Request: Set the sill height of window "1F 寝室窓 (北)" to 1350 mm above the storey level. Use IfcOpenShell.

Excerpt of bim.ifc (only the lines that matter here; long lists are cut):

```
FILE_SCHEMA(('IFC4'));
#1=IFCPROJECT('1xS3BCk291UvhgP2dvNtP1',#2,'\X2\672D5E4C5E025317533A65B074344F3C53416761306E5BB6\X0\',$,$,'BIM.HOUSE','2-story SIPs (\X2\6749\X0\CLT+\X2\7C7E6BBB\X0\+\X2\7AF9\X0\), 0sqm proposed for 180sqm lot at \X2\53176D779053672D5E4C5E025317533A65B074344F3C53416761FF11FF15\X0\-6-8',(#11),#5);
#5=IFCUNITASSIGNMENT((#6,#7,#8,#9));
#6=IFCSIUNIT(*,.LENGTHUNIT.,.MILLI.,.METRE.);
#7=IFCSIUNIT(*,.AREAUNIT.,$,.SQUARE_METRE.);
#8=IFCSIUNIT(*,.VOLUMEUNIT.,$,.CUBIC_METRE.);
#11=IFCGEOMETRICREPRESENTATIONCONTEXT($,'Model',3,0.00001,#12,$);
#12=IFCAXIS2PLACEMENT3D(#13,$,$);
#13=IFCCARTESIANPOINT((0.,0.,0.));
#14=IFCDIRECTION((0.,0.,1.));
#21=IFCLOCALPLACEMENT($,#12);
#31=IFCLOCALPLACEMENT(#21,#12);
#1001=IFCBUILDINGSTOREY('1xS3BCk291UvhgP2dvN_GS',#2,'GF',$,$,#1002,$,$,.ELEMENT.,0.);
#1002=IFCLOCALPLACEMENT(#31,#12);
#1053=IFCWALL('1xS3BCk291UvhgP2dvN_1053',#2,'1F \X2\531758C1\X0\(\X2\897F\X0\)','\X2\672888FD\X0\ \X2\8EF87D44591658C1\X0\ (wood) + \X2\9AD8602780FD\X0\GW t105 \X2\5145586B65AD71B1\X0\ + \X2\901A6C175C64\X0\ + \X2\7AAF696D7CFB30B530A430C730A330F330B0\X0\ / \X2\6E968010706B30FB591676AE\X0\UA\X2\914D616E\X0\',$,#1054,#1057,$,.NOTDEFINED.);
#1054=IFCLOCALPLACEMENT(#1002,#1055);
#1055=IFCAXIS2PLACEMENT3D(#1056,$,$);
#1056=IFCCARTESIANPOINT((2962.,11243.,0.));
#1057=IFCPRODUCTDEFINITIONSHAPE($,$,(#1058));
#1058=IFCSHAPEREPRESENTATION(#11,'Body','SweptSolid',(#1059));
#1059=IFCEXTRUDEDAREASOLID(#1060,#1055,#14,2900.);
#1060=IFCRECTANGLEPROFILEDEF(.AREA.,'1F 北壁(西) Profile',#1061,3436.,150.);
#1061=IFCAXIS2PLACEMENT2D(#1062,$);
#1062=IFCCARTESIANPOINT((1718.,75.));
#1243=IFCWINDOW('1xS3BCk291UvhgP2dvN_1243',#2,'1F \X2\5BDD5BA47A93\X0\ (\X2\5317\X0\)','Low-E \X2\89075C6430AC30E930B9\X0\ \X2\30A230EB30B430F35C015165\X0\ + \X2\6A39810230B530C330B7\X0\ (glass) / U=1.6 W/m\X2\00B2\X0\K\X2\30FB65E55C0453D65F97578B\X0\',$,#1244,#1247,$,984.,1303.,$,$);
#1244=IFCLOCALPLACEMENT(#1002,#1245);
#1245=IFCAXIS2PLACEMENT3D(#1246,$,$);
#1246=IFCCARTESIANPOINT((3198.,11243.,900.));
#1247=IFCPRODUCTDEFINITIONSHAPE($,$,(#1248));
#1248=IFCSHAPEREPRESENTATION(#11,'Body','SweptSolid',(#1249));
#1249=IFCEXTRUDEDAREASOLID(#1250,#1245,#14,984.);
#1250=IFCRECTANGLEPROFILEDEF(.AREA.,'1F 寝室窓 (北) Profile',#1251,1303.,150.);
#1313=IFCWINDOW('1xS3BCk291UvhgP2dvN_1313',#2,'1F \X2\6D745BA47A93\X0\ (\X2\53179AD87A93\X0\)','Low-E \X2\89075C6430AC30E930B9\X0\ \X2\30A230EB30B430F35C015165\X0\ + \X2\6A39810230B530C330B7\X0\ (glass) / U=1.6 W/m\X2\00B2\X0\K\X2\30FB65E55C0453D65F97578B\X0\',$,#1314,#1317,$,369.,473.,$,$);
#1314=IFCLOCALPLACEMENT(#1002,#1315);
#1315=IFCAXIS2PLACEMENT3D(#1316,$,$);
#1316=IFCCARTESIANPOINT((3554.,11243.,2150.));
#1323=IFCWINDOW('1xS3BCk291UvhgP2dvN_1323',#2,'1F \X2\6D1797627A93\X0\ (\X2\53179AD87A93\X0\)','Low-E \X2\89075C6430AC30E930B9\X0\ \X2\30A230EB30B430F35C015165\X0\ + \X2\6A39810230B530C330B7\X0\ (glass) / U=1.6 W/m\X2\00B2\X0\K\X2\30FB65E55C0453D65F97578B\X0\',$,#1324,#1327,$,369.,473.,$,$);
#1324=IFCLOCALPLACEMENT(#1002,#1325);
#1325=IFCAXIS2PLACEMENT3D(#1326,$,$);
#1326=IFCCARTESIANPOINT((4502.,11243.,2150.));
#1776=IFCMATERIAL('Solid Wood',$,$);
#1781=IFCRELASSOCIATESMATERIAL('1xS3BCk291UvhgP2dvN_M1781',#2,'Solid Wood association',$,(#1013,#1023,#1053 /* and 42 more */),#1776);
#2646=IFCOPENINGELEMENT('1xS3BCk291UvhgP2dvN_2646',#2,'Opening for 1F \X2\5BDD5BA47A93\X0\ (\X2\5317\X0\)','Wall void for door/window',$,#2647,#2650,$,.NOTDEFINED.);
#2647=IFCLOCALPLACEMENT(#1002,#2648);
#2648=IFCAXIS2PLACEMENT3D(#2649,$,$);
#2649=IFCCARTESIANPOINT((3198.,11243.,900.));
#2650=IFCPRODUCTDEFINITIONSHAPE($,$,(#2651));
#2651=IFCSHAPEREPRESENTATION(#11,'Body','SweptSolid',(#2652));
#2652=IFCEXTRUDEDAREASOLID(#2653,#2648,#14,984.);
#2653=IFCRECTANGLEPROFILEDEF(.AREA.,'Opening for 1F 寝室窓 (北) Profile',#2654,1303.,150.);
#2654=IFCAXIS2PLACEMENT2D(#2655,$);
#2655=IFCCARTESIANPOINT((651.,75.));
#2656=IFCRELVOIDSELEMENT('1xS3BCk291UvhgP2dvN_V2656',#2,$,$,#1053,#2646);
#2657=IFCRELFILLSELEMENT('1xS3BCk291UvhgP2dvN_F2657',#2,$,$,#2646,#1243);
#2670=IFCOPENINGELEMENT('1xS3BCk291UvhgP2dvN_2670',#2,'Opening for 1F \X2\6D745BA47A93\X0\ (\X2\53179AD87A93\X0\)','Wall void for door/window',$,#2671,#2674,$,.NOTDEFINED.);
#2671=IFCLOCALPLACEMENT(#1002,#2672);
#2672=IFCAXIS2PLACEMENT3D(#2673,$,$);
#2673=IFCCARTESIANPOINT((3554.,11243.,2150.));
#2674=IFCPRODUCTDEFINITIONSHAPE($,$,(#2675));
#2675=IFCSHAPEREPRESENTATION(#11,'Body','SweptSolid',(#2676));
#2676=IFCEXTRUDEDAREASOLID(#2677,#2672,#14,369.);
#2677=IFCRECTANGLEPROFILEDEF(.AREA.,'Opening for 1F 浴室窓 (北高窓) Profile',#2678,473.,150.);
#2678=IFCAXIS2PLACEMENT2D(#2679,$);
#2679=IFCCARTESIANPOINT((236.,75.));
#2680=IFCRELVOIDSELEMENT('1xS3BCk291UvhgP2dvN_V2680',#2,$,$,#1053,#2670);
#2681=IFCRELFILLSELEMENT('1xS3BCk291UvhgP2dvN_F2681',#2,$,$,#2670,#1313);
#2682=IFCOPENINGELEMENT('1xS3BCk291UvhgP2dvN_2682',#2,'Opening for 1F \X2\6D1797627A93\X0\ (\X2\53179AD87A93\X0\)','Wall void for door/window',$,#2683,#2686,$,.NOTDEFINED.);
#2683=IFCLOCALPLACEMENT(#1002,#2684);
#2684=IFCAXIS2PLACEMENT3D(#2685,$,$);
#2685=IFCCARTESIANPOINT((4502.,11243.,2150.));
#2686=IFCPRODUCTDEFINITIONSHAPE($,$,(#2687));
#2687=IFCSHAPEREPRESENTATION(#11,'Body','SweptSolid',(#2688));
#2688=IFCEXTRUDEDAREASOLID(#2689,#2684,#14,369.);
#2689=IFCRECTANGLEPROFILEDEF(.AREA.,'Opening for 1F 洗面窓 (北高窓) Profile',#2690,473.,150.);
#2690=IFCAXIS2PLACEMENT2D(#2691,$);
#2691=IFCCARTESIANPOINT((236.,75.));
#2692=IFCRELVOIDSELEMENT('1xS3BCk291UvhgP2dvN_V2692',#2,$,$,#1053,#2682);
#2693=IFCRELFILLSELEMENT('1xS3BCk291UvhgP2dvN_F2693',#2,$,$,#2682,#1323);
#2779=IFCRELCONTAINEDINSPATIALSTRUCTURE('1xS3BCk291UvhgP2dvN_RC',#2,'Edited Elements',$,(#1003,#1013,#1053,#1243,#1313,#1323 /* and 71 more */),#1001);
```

```python
import numpy as np
import ifcopenshell
import ifcopenshell.api.geometry
import ifcopenshell.geom
import ifcopenshell.util.element
import ifcopenshell.util.placement
import ifcopenshell.util.shape
import ifcopenshell.util.unit

model = ifcopenshell.open("bim.ifc")
unit_scale = ifcopenshell.util.unit.calculate_unit_scale(model)

window = model.by_guid("1xS3BCk291UvhgP2dvN_1243")
opening = window.FillsVoids[0].RelatingOpeningElement
storey = ifcopenshell.util.element.get_container(window, ifc_class="IfcBuildingStorey")
level = ifcopenshell.util.placement.get_local_placement(storey.ObjectPlacement)[2, 3]

# The opening's origin need not be at the sill, so measure its lowest point.
shape = ifcopenshell.geom.create_shape(ifcopenshell.geom.settings(), opening)
bottom = ifcopenshell.util.shape.get_shape_bottom_elevation(shape, shape.geometry) / unit_scale
dz = level + 1.35 / unit_scale - bottom

shift = np.array([0.0, 0.0, dz])
# The window is not placed relative to its opening, so move both.
for product in (opening, window):
    matrix = ifcopenshell.util.placement.get_local_placement(product.ObjectPlacement)
    matrix[:3, 3] += shift
    ifcopenshell.api.geometry.edit_object_placement(model, product=product, matrix=matrix, is_si=False)

print(f"moved by {dz * unit_scale:+.3f} m")

model.write("bim_rev.ifc")
```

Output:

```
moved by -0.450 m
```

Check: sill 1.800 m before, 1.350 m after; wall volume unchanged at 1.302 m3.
